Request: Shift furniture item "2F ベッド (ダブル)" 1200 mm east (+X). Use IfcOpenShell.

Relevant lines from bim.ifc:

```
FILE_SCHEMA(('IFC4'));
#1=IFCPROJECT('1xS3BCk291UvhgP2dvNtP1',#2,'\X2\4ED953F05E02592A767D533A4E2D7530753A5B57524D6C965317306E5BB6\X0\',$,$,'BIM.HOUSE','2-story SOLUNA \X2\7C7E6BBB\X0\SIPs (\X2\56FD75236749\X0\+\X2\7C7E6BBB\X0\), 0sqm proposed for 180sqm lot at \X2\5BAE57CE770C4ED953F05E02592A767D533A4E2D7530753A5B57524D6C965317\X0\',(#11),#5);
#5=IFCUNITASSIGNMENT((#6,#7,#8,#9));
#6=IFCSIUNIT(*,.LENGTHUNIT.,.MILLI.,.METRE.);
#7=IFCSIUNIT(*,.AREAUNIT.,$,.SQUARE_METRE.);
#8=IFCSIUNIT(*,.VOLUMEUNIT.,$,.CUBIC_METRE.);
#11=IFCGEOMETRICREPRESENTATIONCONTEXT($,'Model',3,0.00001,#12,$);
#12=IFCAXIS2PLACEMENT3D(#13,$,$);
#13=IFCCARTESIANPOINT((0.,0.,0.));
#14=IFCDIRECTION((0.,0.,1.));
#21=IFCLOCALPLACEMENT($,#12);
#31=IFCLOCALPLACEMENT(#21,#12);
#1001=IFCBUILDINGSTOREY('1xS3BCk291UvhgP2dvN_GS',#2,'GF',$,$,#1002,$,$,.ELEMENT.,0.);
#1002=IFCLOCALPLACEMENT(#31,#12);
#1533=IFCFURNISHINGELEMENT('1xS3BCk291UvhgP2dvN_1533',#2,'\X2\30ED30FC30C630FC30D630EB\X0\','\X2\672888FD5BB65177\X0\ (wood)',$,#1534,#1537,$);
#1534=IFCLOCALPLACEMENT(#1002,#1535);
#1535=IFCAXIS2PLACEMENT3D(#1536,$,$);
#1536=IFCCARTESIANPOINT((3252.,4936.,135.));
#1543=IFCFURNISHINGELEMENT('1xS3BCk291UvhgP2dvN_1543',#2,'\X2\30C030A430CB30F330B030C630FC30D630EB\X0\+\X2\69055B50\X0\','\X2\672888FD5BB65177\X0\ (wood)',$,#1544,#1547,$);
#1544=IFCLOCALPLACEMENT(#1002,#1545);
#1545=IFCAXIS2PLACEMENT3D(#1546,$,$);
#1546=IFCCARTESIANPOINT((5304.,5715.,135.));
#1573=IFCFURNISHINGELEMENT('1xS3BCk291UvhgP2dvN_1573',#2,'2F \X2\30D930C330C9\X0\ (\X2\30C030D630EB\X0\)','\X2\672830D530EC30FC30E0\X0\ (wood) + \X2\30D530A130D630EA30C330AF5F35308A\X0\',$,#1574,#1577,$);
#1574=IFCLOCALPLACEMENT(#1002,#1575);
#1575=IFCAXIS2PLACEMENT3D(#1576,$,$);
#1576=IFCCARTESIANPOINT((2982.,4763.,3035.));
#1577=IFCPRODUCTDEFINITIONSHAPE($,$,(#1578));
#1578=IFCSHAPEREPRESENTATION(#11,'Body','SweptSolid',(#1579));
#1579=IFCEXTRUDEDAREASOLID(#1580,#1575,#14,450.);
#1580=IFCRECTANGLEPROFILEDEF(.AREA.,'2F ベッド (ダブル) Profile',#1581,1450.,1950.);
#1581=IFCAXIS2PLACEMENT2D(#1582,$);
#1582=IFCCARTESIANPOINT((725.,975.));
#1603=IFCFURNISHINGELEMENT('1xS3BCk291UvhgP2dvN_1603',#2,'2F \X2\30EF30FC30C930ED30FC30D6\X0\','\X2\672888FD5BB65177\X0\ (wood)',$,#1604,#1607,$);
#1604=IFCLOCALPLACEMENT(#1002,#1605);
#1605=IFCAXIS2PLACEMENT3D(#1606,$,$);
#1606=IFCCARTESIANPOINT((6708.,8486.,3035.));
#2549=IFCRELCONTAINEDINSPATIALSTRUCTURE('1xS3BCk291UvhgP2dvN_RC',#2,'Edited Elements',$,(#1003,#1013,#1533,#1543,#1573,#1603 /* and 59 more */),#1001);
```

```python
import ifcopenshell
import ifcopenshell.api.geometry
import ifcopenshell.util.placement
import ifcopenshell.util.unit

model = ifcopenshell.open("bim.ifc")
unit_scale = ifcopenshell.util.unit.calculate_unit_scale(model)

item = model.by_id(1573)
matrix = ifcopenshell.util.placement.get_local_placement(item.ObjectPlacement)
matrix[0, 3] += 1.2 / unit_scale
ifcopenshell.api.geometry.edit_object_placement(model, product=item, matrix=matrix, is_si=False)

print(ifcopenshell.util.placement.get_local_placement(item.ObjectPlacement).round(3) + 0.0)

model.write("bim_edited.ifc")
```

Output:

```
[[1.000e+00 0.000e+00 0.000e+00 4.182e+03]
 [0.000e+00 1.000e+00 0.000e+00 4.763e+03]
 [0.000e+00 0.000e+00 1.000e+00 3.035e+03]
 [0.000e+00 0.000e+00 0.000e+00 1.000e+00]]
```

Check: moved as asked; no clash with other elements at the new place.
